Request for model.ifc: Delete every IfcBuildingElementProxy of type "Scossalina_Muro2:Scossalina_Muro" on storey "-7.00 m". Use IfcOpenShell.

First a look at what the model holds.

```python
import ifcopenshell
import ifcopenshell.util.element

model = ifcopenshell.open("model.ifc")
print(model.schema)
storey = next(s for s in model.by_type("IfcBuildingStorey") if s.Name == "-7.00 m")
proxies = [e for e in ifcopenshell.util.element.get_decomposition(storey) if e.is_a("IfcBuildingElementProxy")]
seen = {}
for e in proxies:
    element_type = ifcopenshell.util.element.get_type(e)
    name = element_type.Name if element_type not in (None, e) else None
    seen[name] = seen.get(name, 0) + 1
for name, count in sorted(seen.items(), key=str):
    print(count, "x", name)
```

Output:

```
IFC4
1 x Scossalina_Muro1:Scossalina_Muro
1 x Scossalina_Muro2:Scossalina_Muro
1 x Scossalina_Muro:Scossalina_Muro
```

```python
import ifcopenshell
import ifcopenshell.api.root
import ifcopenshell.util.element

model = ifcopenshell.open("model.ifc")

storey = next(s for s in model.by_type("IfcBuildingStorey") if s.Name == "-7.00 m")
proxies = [e for e in ifcopenshell.util.element.get_decomposition(storey) if e.is_a("IfcBuildingElementProxy")]
targets = [e for e in proxies if (t := ifcopenshell.util.element.get_type(e)) not in (None, e) and t.Name == "Scossalina_Muro2:Scossalina_Muro"]

for e in targets:
    ifcopenshell.api.root.remove_product(model, product=e)
print(len(targets), "removed")

model.write("model_v2.ifc")
```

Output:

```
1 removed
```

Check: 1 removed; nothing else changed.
